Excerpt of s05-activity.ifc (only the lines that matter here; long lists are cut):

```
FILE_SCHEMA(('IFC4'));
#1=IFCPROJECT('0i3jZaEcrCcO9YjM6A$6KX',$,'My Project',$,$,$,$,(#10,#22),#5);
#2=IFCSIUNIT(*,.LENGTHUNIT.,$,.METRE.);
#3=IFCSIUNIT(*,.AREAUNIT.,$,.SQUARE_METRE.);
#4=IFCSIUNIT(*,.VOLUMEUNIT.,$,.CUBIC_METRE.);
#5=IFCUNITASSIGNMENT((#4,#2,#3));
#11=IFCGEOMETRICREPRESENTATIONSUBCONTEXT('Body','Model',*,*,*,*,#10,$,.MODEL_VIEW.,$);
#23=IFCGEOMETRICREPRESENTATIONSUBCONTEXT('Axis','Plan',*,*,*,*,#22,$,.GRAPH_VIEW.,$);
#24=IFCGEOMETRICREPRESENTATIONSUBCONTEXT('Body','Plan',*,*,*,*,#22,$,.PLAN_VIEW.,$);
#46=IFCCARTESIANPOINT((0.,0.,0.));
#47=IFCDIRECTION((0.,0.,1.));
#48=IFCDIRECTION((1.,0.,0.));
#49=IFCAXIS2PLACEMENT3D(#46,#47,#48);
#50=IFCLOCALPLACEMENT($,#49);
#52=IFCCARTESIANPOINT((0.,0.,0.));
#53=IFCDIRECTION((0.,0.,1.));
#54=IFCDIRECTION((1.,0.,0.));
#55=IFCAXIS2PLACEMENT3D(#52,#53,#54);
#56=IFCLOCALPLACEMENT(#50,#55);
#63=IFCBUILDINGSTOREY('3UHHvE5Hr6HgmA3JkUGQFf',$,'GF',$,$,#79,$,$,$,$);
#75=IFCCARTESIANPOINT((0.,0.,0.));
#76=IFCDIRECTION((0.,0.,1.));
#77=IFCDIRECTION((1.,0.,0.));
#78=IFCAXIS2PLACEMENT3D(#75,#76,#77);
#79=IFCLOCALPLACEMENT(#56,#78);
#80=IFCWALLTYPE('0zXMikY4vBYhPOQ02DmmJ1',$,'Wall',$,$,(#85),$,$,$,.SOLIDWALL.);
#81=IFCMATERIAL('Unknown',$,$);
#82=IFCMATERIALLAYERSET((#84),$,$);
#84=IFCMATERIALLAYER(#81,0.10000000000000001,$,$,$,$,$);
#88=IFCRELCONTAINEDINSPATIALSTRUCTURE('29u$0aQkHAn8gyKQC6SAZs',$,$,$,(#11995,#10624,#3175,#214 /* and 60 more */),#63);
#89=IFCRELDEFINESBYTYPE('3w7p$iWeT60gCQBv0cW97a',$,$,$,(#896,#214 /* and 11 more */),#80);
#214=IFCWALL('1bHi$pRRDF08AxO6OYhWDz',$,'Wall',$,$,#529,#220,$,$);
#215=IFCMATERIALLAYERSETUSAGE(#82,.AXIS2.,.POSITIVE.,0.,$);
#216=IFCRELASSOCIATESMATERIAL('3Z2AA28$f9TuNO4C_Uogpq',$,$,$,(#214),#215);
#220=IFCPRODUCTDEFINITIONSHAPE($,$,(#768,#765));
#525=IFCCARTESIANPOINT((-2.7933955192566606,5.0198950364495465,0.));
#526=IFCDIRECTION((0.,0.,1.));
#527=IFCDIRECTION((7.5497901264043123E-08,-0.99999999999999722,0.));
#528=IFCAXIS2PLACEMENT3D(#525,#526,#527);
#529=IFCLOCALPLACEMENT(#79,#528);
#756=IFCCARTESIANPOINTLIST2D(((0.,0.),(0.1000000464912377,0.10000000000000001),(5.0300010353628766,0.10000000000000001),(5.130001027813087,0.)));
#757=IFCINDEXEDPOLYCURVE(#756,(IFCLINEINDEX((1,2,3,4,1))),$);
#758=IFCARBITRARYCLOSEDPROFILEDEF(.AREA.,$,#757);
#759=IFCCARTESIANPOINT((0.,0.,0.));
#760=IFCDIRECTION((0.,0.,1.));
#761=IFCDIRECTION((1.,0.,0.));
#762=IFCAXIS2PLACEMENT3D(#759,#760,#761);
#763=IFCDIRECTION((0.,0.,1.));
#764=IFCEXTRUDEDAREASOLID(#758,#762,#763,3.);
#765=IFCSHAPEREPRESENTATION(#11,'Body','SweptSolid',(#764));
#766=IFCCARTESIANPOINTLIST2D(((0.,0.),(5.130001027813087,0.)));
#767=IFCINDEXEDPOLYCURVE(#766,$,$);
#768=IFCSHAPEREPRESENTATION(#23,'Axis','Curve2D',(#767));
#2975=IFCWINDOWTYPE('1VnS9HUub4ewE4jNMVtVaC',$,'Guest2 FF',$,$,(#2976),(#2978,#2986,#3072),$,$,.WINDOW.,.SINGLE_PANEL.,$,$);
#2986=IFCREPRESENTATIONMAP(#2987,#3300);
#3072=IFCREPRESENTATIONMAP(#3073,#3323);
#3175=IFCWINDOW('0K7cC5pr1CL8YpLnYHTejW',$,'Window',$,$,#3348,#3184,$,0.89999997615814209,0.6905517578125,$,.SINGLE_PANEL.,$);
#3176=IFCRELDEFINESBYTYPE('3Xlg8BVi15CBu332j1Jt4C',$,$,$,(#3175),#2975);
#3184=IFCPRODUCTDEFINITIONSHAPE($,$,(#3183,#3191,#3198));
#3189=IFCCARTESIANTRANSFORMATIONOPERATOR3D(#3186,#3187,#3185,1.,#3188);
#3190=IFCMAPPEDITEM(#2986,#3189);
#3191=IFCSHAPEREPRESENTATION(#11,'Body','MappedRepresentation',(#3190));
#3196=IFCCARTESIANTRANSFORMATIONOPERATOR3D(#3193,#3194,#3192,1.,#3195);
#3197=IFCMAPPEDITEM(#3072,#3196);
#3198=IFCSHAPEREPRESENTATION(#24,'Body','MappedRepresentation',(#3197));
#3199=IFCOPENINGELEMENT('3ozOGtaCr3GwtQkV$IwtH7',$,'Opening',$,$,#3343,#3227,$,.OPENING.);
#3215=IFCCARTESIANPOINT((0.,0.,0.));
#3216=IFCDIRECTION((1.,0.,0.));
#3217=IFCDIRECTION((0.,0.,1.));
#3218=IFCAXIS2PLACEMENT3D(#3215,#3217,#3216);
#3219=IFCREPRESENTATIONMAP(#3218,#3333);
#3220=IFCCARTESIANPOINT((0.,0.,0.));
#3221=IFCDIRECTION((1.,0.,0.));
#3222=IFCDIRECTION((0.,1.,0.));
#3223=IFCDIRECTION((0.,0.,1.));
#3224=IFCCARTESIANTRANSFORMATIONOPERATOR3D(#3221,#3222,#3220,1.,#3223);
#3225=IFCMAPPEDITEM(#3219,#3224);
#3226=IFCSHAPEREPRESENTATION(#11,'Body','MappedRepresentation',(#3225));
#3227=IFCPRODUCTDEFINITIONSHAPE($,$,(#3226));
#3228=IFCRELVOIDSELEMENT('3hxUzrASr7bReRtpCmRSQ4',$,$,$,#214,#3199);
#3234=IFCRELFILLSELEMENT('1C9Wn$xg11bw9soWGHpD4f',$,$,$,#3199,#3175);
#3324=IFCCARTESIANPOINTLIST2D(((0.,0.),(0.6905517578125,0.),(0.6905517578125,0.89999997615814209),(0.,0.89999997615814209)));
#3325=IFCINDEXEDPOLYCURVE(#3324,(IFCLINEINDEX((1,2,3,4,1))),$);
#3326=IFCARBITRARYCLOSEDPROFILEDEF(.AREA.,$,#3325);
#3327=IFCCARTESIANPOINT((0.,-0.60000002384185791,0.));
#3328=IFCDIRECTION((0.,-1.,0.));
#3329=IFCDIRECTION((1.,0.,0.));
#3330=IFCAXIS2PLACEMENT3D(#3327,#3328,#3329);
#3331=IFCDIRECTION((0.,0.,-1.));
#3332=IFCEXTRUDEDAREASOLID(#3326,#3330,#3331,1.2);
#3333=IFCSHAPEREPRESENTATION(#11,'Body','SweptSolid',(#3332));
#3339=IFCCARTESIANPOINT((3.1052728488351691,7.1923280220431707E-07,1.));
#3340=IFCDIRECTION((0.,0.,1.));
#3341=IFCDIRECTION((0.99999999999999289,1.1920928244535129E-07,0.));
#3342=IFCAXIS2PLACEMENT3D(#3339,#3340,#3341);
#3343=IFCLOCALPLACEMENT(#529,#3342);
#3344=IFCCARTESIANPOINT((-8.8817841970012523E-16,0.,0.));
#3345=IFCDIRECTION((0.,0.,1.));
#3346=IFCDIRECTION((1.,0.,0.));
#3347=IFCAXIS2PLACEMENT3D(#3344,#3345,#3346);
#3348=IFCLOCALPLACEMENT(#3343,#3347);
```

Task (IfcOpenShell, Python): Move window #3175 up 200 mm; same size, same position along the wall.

```python
import numpy as np
import ifcopenshell
import ifcopenshell.api.geometry
import ifcopenshell.util.placement
import ifcopenshell.util.unit

model = ifcopenshell.open("s05-activity.ifc")
unit_scale = ifcopenshell.util.unit.calculate_unit_scale(model)

window = model.by_id(3175)
opening = window.FillsVoids[0].RelatingOpeningElement
dz = 0.2 / unit_scale

shift = np.array([0.0, 0.0, dz])
# The window is placed relative to its opening, so it follows when the opening moves.
matrix = ifcopenshell.util.placement.get_local_placement(opening.ObjectPlacement)
matrix[:3, 3] += shift
ifcopenshell.api.geometry.edit_object_placement(
    model, product=opening, matrix=matrix, is_si=False, should_transform_children=True
)

print(f"moved by {dz * unit_scale:+.3f} m")

model.write("s05-activity_v2.ifc")
```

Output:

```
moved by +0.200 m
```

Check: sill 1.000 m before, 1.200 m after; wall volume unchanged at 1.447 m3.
